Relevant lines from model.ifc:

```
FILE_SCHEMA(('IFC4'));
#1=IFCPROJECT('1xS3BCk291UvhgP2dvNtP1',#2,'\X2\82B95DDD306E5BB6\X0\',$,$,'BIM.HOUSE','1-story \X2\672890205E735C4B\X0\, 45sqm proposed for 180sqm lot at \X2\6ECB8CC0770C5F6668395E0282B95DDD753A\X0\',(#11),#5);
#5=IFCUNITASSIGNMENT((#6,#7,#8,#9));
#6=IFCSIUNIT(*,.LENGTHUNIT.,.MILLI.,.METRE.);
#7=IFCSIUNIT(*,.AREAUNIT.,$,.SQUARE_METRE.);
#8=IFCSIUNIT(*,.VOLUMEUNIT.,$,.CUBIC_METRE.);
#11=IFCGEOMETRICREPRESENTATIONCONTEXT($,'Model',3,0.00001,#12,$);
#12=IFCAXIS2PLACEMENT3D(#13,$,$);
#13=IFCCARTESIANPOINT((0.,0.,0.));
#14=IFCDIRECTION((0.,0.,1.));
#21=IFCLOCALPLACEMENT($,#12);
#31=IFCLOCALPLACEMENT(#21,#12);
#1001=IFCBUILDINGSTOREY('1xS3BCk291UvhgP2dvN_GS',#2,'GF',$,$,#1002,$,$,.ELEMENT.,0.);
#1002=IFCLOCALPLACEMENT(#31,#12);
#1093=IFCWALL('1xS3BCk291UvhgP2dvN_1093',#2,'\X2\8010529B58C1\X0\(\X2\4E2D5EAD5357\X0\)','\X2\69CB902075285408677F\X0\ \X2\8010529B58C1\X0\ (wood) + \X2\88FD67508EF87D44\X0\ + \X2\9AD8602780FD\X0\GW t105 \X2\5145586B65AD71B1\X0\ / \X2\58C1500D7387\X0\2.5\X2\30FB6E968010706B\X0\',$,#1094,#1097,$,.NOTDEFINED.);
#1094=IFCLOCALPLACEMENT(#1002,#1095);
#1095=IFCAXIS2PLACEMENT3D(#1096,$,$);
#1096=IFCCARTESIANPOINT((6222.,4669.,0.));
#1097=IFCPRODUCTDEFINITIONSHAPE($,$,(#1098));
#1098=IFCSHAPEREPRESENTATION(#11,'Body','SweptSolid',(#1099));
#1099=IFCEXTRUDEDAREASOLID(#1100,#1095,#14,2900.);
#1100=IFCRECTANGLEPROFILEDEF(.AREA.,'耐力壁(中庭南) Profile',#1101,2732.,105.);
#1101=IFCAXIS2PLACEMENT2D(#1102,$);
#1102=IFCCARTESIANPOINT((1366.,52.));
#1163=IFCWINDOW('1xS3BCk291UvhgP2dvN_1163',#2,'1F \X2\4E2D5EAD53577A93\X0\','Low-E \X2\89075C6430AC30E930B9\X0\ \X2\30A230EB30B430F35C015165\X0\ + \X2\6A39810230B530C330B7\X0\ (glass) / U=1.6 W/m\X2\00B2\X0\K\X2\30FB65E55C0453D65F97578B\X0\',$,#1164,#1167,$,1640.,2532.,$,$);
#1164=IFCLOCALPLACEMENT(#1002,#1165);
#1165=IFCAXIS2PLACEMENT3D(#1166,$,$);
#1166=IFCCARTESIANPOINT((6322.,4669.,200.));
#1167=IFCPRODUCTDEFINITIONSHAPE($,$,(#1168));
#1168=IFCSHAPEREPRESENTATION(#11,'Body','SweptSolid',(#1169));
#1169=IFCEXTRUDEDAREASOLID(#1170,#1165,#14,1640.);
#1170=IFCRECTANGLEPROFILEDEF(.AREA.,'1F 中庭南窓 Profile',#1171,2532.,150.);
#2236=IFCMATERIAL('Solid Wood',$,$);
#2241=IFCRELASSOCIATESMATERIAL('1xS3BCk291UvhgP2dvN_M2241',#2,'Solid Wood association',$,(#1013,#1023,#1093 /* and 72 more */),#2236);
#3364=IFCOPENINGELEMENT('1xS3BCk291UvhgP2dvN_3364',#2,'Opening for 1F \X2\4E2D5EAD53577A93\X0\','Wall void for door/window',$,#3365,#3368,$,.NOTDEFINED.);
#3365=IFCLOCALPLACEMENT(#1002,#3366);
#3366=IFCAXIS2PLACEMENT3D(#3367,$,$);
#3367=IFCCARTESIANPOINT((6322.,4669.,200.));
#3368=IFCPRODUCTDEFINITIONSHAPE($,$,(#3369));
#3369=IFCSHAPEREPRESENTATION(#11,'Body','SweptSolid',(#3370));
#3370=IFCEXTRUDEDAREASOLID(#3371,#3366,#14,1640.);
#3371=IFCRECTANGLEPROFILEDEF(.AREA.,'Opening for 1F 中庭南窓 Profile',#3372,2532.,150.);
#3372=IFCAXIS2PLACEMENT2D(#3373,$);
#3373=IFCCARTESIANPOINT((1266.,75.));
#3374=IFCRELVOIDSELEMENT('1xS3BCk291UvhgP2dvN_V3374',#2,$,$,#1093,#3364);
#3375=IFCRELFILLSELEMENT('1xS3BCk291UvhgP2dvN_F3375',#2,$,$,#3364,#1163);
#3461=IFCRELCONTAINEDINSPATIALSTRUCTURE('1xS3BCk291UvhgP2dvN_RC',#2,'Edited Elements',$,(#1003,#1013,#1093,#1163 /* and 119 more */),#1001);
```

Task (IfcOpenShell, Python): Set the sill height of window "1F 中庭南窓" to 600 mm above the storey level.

```python
import numpy as np
import ifcopenshell
import ifcopenshell.api.geometry
import ifcopenshell.geom
import ifcopenshell.util.element
import ifcopenshell.util.placement
import ifcopenshell.util.shape
import ifcopenshell.util.unit

model = ifcopenshell.open("model.ifc")
unit_scale = ifcopenshell.util.unit.calculate_unit_scale(model)

window = model.by_id(1163)
opening = window.FillsVoids[0].RelatingOpeningElement
storey = ifcopenshell.util.element.get_container(window, ifc_class="IfcBuildingStorey")
level = ifcopenshell.util.placement.get_local_placement(storey.ObjectPlacement)[2, 3]

# The opening's origin need not be at the sill, so measure its lowest point.
shape = ifcopenshell.geom.create_shape(ifcopenshell.geom.settings(), opening)
bottom = ifcopenshell.util.shape.get_shape_bottom_elevation(shape, shape.geometry) / unit_scale
dz = level + 0.6 / unit_scale - bottom

shift = np.array([0.0, 0.0, dz])
# The window is not placed relative to its opening, so move both.
for product in (opening, window):
    matrix = ifcopenshell.util.placement.get_local_placement(product.ObjectPlacement)
    matrix[:3, 3] += shift
    ifcopenshell.api.geometry.edit_object_placement(model, product=product, matrix=matrix, is_si=False)

print(f"moved by {dz * unit_scale:+.3f} m")

model.write("model_rev.ifc")
```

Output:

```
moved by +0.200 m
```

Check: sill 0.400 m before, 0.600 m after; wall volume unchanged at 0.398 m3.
